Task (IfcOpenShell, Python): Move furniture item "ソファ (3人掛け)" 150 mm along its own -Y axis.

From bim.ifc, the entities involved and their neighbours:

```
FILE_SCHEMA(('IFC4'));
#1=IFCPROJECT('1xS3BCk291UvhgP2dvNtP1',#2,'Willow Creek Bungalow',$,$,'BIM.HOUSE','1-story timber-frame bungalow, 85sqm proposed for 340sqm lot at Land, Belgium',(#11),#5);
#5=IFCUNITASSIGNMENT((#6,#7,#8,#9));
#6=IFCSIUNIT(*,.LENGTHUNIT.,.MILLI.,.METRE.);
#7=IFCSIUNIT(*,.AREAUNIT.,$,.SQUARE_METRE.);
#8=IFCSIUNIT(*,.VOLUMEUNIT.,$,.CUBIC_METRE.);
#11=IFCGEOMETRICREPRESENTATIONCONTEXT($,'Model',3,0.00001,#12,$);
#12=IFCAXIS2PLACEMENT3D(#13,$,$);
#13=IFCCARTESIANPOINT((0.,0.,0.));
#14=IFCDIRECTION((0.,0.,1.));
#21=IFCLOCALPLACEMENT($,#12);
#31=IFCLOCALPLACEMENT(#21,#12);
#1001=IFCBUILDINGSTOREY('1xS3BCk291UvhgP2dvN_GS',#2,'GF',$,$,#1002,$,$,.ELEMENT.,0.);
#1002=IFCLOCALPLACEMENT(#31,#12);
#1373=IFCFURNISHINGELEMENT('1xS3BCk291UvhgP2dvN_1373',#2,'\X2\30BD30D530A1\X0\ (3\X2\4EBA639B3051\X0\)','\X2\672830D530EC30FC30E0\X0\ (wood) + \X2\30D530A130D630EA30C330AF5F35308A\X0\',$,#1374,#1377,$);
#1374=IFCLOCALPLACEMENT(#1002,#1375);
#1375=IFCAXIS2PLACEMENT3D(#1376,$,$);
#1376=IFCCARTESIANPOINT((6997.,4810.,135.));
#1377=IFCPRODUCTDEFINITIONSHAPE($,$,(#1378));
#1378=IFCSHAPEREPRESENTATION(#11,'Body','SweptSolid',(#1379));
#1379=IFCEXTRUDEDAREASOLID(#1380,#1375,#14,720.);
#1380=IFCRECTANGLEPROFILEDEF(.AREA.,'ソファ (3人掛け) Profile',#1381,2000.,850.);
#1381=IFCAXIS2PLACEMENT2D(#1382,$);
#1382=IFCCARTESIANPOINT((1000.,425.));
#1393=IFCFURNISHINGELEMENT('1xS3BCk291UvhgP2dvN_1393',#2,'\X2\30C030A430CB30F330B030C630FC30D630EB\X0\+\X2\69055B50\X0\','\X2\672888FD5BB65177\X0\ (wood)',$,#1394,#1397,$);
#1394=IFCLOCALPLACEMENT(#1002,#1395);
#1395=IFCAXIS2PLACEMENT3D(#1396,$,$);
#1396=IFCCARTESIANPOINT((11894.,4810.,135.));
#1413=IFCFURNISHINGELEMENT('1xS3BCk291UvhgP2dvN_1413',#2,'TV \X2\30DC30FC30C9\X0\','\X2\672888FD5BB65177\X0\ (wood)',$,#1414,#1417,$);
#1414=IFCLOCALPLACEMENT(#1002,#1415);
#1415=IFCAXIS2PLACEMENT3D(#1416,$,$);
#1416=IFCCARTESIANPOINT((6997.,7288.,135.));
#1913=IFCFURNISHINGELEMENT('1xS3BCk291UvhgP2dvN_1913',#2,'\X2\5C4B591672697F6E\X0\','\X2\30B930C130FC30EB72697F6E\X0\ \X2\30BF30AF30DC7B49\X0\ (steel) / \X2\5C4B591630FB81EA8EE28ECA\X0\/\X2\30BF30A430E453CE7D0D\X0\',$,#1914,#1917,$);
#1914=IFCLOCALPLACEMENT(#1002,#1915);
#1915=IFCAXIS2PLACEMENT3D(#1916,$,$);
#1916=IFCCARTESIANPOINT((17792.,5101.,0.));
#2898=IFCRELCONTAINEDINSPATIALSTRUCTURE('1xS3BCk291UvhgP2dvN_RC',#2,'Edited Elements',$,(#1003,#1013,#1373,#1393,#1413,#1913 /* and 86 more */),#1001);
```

```python
import ifcopenshell
import ifcopenshell.api.geometry
import ifcopenshell.util.placement
import ifcopenshell.util.unit

model = ifcopenshell.open("bim.ifc")
unit_scale = ifcopenshell.util.unit.calculate_unit_scale(model)

item = model.by_guid("1xS3BCk291UvhgP2dvN_1373")
matrix = ifcopenshell.util.placement.get_local_placement(item.ObjectPlacement)
matrix[:3, 3] -= matrix[:3, 1] * 0.15 / unit_scale
ifcopenshell.api.geometry.edit_object_placement(model, product=item, matrix=matrix, is_si=False)

print(ifcopenshell.util.placement.get_local_placement(item.ObjectPlacement).round(3) + 0.0)

model.write("bim_updated.ifc")
```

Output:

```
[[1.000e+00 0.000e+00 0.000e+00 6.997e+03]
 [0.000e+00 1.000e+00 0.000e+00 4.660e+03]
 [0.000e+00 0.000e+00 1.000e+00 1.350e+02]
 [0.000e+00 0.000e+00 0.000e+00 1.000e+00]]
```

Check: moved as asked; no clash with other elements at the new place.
